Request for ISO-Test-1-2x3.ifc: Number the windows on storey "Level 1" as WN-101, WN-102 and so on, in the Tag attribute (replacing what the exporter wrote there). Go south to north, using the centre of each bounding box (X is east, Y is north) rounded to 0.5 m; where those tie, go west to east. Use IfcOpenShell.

First a look at what the model holds.

```python
import ifcopenshell
import ifcopenshell.util.element
import ifcopenshell.util.placement

model = ifcopenshell.open("ISO-Test-1-2x3.ifc")
print(model.schema)
storey = next(s for s in model.by_type("IfcBuildingStorey") if s.Name == "Level 1")
windows = [e for e in ifcopenshell.util.element.get_decomposition(storey) if e.is_a("IfcWindow")]
for e in sorted(windows, key=lambda e: e.id()):
    origin = ifcopenshell.util.placement.get_local_placement(e.ObjectPlacement)[:3, 3]
    print(e.id(), e.Tag, e.Name, origin.round(2) + 0.0, sep=" | ")
```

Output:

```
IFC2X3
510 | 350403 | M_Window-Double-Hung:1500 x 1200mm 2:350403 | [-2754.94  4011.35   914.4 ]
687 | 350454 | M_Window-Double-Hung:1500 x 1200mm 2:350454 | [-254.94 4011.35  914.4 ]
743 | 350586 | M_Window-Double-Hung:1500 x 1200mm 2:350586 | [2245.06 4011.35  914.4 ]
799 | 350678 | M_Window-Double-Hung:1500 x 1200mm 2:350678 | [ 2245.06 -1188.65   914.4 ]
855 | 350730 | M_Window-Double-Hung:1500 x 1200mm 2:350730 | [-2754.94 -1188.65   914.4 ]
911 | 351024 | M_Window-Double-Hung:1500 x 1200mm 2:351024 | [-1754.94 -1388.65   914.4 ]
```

```python
import ifcopenshell
import ifcopenshell.geom
import ifcopenshell.util.element
import ifcopenshell.util.shape

model = ifcopenshell.open("ISO-Test-1-2x3.ifc")
settings = ifcopenshell.geom.settings()
settings.set("use-world-coords", True)


def centre(element):
    shape = ifcopenshell.geom.create_shape(settings, element)
    return ifcopenshell.util.shape.get_bbox_centroid(shape.geometry)


storey = next(s for s in model.by_type("IfcBuildingStorey") if s.Name == "Level 1")
windows = [e for e in ifcopenshell.util.element.get_decomposition(storey) if e.is_a("IfcWindow")]

# Insertion points can sit at a corner or the storey origin, so sort by the geometry (in metres).
centres = {e: centre(e) for e in windows}
windows.sort(key=lambda e: (round(centres[e][1] / 0.5), centres[e][0]))

for i, e in enumerate(windows, start=1):
    number = f"WN-1{i:02d}"
    e.Tag = number
    print(e.id(), number)

model.write("ISO-Test-1-2x3_updated.ifc")
```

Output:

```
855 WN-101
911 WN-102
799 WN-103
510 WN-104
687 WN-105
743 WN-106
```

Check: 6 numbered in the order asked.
